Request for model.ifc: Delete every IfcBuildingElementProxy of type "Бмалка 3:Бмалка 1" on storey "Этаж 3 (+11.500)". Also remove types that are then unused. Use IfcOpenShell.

First a look at what the model holds.

```python
import ifcopenshell
import ifcopenshell.util.element

model = ifcopenshell.open("model.ifc")
print(model.schema)
storey = next(s for s in model.by_type("IfcBuildingStorey") if s.Name == "Этаж 3 (+11.500)")
proxies = [e for e in ifcopenshell.util.element.get_decomposition(storey) if e.is_a("IfcBuildingElementProxy")]
seen = {}
for e in proxies:
    element_type = ifcopenshell.util.element.get_type(e)
    name = element_type.Name if element_type not in (None, e) else None
    seen[name] = seen.get(name, 0) + 1
for name, count in sorted(seen.items(), key=str):
    print(count, "x", name)
```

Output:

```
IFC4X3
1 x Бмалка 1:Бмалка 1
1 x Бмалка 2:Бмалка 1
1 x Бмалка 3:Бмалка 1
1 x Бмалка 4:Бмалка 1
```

```python
import ifcopenshell
import ifcopenshell.api.root
import ifcopenshell.util.element

model = ifcopenshell.open("model.ifc")

storey = next(s for s in model.by_type("IfcBuildingStorey") if s.Name == "Этаж 3 (+11.500)")
proxies = [e for e in ifcopenshell.util.element.get_decomposition(storey) if e.is_a("IfcBuildingElementProxy")]
targets = [e for e in proxies if (t := ifcopenshell.util.element.get_type(e)) not in (None, e) and t.Name == "Бмалка 3:Бмалка 1"]
types = {ifcopenshell.util.element.get_type(e) for e in targets} - {None, *targets}

for e in targets:
    ifcopenshell.api.root.remove_product(model, product=e)
print(len(targets), "removed")

unused = [t for t in types if not ifcopenshell.util.element.get_types(t)]
for t in unused:
    ifcopenshell.api.root.remove_product(model, product=t)
print(len(unused), "unused types removed")

model.write("model_rev.ifc")
```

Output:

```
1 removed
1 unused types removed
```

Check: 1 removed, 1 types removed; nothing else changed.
